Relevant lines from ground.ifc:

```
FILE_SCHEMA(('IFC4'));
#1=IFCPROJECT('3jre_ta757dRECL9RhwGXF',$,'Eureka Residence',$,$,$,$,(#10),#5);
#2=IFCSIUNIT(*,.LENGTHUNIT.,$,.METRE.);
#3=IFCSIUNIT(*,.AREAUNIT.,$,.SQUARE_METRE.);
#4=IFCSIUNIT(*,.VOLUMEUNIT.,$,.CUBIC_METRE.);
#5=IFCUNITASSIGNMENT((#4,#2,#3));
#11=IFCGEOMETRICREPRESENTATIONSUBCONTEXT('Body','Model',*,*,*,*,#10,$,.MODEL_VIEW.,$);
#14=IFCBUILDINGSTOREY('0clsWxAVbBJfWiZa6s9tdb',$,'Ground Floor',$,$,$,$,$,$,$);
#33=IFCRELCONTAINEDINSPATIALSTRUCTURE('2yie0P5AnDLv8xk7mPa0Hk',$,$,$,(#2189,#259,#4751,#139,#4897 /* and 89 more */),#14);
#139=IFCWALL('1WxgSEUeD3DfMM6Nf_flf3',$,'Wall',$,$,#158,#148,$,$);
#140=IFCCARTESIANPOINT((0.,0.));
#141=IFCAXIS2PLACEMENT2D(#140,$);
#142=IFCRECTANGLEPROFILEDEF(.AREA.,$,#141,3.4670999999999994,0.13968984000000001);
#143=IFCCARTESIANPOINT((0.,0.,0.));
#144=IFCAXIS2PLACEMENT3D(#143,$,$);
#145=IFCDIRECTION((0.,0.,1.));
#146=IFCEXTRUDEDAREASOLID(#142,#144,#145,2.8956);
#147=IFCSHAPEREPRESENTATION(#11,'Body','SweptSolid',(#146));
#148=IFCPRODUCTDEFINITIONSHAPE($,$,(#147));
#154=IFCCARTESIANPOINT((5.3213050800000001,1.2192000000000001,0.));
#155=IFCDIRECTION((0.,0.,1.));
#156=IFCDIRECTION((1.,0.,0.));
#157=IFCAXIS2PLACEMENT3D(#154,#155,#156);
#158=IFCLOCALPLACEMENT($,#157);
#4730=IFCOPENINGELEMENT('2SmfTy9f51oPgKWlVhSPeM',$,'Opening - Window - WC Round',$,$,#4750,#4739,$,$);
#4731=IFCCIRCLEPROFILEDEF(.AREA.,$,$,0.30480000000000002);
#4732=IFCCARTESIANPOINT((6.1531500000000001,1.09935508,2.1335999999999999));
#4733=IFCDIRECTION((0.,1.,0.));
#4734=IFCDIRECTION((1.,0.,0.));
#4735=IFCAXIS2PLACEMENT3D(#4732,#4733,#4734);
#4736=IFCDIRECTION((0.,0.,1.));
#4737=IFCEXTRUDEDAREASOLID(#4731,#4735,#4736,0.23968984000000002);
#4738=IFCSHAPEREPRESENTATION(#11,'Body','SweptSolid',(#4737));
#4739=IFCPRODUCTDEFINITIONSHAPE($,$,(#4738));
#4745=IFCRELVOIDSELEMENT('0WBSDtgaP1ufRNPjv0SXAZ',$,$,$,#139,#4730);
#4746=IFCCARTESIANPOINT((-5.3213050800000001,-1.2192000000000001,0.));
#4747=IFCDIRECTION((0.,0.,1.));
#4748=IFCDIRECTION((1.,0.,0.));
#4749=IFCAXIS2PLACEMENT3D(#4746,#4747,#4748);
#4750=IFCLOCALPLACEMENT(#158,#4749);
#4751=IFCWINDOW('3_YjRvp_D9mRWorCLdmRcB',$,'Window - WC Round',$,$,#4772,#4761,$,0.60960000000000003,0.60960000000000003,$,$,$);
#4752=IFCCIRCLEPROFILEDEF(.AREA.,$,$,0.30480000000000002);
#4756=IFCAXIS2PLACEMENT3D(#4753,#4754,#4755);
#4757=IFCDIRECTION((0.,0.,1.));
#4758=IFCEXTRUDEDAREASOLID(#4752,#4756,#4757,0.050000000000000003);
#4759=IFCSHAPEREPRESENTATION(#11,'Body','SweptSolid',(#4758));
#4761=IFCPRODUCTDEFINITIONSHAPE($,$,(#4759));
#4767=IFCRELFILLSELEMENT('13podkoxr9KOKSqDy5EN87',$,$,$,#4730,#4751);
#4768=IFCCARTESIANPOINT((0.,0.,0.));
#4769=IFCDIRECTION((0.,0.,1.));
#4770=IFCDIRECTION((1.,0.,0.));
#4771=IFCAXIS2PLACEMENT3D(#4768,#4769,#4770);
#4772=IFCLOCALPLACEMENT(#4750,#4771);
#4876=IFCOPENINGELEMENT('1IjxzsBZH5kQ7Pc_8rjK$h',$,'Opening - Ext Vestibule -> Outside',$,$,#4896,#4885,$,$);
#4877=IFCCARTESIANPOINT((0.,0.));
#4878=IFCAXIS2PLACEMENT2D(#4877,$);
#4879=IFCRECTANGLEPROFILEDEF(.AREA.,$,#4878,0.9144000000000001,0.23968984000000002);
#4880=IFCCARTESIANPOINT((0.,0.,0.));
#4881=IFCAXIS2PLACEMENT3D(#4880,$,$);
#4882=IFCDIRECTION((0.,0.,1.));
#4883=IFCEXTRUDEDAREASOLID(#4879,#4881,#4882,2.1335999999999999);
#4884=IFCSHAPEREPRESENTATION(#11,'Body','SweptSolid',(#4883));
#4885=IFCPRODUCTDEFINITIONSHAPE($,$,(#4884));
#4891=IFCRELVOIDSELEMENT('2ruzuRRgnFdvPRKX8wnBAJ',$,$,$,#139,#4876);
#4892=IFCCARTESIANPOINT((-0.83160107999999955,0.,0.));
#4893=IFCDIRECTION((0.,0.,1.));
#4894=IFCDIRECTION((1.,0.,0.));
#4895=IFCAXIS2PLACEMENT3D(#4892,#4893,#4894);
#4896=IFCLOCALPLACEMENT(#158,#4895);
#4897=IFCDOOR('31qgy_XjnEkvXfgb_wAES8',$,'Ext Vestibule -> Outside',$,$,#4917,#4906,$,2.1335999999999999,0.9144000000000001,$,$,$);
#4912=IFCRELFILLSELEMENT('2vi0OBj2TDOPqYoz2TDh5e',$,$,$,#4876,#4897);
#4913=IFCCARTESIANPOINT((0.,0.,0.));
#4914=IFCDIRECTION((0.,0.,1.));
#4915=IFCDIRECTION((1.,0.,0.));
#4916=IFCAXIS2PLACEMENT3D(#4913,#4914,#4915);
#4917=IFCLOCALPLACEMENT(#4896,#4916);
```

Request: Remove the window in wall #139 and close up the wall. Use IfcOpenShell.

```python
import ifcopenshell
import ifcopenshell.api.feature
import ifcopenshell.api.root
import ifcopenshell.geom
import ifcopenshell.util.shape

model = ifcopenshell.open("ground.ifc")
settings = ifcopenshell.geom.settings()


def volume(element):
    """Net volume in cubic metres, openings subtracted."""
    shape = ifcopenshell.geom.create_shape(settings, element)
    return ifcopenshell.util.shape.get_volume(shape.geometry)


window = model.by_id(4751)
opening = window.FillsVoids[0].RelatingOpeningElement
wall = opening.VoidsElements[0].RelatingBuildingElement
before = volume(wall)

ifcopenshell.api.root.remove_product(model, product=window)
ifcopenshell.api.feature.remove_feature(model, feature=opening)

after = volume(wall)

print(f"wall volume {before:.3f} -> {after:.3f} m3")

model.write("ground_v2.ifc")
```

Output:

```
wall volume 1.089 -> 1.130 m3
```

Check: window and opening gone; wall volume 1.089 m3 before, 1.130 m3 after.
